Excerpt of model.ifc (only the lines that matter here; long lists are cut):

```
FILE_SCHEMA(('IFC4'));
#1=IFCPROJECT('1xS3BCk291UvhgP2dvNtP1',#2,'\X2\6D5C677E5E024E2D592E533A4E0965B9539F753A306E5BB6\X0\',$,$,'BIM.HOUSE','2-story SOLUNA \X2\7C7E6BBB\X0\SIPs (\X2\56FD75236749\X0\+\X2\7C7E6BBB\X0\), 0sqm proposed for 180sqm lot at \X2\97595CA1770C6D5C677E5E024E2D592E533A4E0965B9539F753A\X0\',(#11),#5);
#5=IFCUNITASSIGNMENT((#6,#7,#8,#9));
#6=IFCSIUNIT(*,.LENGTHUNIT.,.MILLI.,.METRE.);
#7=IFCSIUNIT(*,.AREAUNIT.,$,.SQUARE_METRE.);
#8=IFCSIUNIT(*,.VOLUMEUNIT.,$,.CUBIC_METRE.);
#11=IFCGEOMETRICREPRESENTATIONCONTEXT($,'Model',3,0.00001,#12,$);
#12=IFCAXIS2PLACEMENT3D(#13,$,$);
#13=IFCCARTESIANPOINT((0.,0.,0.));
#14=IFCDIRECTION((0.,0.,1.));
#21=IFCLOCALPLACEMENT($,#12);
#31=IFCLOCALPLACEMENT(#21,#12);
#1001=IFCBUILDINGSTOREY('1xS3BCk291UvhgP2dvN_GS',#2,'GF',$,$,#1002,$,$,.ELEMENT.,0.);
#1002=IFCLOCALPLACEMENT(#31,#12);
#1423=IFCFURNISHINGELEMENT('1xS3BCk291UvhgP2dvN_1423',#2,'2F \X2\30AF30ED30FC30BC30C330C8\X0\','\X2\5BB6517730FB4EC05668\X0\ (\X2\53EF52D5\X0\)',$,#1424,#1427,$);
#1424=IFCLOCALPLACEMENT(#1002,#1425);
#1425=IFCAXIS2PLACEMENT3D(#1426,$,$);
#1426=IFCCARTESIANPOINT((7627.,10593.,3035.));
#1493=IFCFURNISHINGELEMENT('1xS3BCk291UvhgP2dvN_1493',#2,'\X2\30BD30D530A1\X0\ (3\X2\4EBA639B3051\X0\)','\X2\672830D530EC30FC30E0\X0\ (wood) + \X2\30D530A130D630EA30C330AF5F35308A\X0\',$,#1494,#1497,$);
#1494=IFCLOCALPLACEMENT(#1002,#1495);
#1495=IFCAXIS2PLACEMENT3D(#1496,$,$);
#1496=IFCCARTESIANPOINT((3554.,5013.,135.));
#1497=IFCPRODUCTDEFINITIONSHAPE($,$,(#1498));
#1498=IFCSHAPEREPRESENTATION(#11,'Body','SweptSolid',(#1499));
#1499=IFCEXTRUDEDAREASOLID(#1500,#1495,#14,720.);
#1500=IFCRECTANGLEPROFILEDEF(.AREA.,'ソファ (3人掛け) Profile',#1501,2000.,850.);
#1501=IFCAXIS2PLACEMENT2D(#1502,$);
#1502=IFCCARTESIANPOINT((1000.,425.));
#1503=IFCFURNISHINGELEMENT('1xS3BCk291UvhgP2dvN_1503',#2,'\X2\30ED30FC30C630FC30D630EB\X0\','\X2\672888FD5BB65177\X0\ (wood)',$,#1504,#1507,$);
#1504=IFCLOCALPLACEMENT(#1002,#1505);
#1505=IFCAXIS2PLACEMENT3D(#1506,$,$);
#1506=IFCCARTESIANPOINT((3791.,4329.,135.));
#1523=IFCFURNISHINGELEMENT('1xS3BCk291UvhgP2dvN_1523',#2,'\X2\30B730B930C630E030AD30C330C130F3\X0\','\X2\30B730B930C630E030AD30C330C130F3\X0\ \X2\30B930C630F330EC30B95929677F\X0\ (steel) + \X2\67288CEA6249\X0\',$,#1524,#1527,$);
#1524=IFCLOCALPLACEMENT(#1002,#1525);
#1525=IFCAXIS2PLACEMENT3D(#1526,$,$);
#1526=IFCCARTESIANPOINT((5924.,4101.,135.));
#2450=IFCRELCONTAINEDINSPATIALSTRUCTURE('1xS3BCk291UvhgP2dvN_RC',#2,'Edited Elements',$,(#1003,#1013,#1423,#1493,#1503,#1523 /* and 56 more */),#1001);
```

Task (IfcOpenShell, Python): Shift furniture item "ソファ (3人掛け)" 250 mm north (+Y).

```python
import ifcopenshell
import ifcopenshell.api.geometry
import ifcopenshell.util.placement
import ifcopenshell.util.unit

model = ifcopenshell.open("model.ifc")
unit_scale = ifcopenshell.util.unit.calculate_unit_scale(model)

item = model.by_id(1493)
matrix = ifcopenshell.util.placement.get_local_placement(item.ObjectPlacement)
matrix[1, 3] += 0.25 / unit_scale
ifcopenshell.api.geometry.edit_object_placement(model, product=item, matrix=matrix, is_si=False)

print(ifcopenshell.util.placement.get_local_placement(item.ObjectPlacement).round(3) + 0.0)

model.write("model_updated.ifc")
```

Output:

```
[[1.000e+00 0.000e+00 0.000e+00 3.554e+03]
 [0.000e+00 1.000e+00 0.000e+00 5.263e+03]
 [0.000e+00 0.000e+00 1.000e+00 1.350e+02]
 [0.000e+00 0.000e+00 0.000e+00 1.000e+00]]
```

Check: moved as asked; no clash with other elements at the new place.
